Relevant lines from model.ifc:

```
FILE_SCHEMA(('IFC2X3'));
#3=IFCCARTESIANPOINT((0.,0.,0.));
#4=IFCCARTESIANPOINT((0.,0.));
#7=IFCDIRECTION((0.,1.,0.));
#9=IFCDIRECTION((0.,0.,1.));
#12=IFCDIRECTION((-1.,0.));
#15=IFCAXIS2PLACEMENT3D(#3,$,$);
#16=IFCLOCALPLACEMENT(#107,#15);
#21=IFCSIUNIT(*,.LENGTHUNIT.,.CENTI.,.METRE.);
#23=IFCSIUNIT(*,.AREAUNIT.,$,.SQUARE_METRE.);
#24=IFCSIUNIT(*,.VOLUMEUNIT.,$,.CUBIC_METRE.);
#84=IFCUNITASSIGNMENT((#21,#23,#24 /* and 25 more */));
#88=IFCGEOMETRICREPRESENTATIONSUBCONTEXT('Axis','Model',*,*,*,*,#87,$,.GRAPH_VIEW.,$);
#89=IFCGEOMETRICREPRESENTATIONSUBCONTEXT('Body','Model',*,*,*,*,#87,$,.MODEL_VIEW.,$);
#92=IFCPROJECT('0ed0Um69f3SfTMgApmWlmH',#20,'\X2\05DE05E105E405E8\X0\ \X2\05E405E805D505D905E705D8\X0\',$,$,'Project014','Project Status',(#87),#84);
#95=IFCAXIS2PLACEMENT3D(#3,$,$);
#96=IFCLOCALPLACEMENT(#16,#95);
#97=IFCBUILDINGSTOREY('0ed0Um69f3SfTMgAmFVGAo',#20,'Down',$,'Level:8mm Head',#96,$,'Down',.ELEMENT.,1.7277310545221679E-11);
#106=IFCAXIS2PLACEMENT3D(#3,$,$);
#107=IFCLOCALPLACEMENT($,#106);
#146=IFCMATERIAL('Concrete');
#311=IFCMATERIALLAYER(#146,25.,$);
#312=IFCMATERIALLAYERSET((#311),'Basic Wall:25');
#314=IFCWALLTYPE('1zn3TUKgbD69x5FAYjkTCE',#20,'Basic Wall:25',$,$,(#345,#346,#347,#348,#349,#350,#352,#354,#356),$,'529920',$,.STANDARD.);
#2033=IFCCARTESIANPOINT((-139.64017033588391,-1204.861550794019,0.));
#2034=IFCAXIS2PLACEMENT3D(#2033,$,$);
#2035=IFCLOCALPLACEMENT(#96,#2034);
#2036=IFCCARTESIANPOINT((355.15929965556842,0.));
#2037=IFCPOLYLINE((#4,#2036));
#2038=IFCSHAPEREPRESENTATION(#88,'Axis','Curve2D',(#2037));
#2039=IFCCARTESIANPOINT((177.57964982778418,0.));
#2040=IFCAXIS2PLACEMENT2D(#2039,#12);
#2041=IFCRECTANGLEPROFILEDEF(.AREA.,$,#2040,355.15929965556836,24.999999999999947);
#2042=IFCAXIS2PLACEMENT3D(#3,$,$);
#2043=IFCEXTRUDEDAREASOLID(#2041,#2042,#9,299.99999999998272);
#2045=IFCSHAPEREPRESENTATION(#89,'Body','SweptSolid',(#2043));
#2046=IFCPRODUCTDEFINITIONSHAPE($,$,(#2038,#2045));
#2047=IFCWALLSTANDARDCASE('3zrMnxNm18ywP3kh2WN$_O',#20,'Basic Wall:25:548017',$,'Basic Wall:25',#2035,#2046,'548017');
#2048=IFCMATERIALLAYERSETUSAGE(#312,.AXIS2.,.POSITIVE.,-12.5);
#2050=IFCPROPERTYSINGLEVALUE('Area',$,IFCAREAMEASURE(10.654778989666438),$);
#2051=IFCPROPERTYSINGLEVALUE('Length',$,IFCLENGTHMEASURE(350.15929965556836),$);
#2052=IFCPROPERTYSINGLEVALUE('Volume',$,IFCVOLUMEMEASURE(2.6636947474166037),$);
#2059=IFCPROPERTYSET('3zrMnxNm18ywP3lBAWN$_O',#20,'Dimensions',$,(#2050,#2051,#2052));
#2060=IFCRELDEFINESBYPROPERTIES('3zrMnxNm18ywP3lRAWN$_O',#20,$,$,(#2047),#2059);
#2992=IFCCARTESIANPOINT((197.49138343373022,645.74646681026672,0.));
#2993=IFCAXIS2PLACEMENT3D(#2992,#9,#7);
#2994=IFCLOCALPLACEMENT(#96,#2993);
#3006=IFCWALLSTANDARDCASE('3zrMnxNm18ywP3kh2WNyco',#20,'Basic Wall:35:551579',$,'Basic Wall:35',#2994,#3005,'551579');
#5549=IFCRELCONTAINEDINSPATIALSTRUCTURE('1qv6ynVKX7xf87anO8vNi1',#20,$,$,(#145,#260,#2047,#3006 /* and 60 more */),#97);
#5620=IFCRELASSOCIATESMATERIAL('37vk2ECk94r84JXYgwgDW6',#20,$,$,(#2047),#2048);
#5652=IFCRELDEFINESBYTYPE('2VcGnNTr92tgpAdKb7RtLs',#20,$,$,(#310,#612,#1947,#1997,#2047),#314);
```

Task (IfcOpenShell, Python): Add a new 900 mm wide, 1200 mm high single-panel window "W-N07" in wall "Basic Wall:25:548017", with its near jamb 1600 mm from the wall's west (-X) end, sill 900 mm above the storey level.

```python
import numpy as np
import ifcopenshell
import ifcopenshell.api.feature
import ifcopenshell.api.geometry
import ifcopenshell.api.pset
import ifcopenshell.api.root
import ifcopenshell.api.spatial
import ifcopenshell.api.type
import ifcopenshell.geom
import ifcopenshell.util.element
import ifcopenshell.util.placement
import ifcopenshell.util.representation
import ifcopenshell.util.shape
import ifcopenshell.util.unit

model = ifcopenshell.open("model.ifc")
unit_scale = ifcopenshell.util.unit.calculate_unit_scale(model)
area_scale = ifcopenshell.util.unit.calculate_unit_scale(model, "AREAUNIT")
volume_scale = ifcopenshell.util.unit.calculate_unit_scale(model, "VOLUMEUNIT")
settings = ifcopenshell.geom.settings()


def volume(element):
    """Net volume in cubic metres, openings subtracted."""
    shape = ifcopenshell.geom.create_shape(settings, element)
    return ifcopenshell.util.shape.get_volume(shape.geometry)


wall = model.by_id(2047)
storey = ifcopenshell.util.element.get_container(wall, ifc_class="IfcBuildingStorey")
context = ifcopenshell.util.representation.get_context(model, "Model", "Body", "MODEL_VIEW")
before = volume(wall)

width, height, from_end, sill = 0.9, 1.2, 1.6, 0.9  # metres

# The wall runs along its own X axis, and the end named is its -X end.
wall_shape = ifcopenshell.geom.create_shape(settings, wall)
x, y, z = ifcopenshell.util.shape.get_vertices(wall_shape.geometry).T
start = x.min() + from_end
face, thickness = float(y.min()), float(y.max() - y.min())
wall_matrix = ifcopenshell.util.placement.get_local_placement(wall.ObjectPlacement)
level = ifcopenshell.util.placement.get_local_placement(storey.ObjectPlacement)[2, 3]


def in_wall(x, y):
    """Placement at x, y metres in the wall's axes, at sill height."""
    matrix = wall_matrix.copy()
    matrix[:, 3] = wall_matrix @ np.array([x / unit_scale, y / unit_scale, 0.0, 1.0])
    matrix[2, 3] = level + sill / unit_scale
    return matrix


# Opening: a box that overshoots both wall faces by 50 mm.
opening = ifcopenshell.api.root.create_entity(model, ifc_class="IfcOpeningElement")
box = ifcopenshell.api.geometry.add_wall_representation(
    model, context=context, length=width, height=height, thickness=thickness + 0.1
)
ifcopenshell.api.geometry.assign_representation(model, product=opening, representation=box)
ifcopenshell.api.geometry.edit_object_placement(model, product=opening, matrix=in_wall(start, face - 0.05), is_si=False)
ifcopenshell.api.feature.add_feature(model, feature=opening, element=wall)

window = ifcopenshell.api.root.create_entity(model, ifc_class="IfcWindow", name="W-N07")
window.OverallWidth, window.OverallHeight = width / unit_scale, height / unit_scale
body = ifcopenshell.api.geometry.add_window_representation(
    model,
    context=context,
    overall_width=window.OverallWidth,
    overall_height=window.OverallHeight,
    partition_type="SINGLE_PANEL",
)
ifcopenshell.api.geometry.assign_representation(model, product=window, representation=body)
ifcopenshell.api.spatial.assign_container(model, products=[window], relating_structure=storey)
fills = ifcopenshell.api.feature.add_filling(model, opening=opening, element=window)
fills.OwnerHistory = window.OwnerHistory  # required in IFC2X3

# IFC2X3 keeps the operation on the window style.
style = ifcopenshell.api.root.create_entity(model, ifc_class="IfcWindowStyle", name="W-N07")
style.OperationType, style.ConstructionType = "SINGLE_PANEL", "NOTDEFINED"
style.ParameterTakesPrecedence = style.Sizeable = False
ifcopenshell.api.type.assign_type(model, related_objects=[window], relating_type=style)

# Centre the window in the wall's thickness.
ifcopenshell.api.geometry.edit_object_placement(model, product=window, matrix=in_wall(start, face), is_si=False)
window_shape = ifcopenshell.geom.create_shape(settings, window)
depth = ifcopenshell.util.shape.get_vertices(window_shape.geometry)[:, 1]
offset = face + thickness / 2 - (depth.min() + depth.max()) / 2
ifcopenshell.api.geometry.edit_object_placement(model, product=window, matrix=in_wall(start, offset), is_si=False)

after = volume(wall)

# Update the wall's stored quantities.
pset = model.by_id(ifcopenshell.util.element.get_pset(wall, "Dimensions", should_inherit=False)["id"])
ifcopenshell.api.pset.edit_pset(model, pset=pset, properties={
    "Area": model.create_entity("IfcAreaMeasure", after / thickness / area_scale),
    "Volume": model.create_entity("IfcVolumeMeasure", after / volume_scale),
})

print(f"wall volume {before:.3f} -> {after:.3f} m3")

model.write("model_v2.ifc")
```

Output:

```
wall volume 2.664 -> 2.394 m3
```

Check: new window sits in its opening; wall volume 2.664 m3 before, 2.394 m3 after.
